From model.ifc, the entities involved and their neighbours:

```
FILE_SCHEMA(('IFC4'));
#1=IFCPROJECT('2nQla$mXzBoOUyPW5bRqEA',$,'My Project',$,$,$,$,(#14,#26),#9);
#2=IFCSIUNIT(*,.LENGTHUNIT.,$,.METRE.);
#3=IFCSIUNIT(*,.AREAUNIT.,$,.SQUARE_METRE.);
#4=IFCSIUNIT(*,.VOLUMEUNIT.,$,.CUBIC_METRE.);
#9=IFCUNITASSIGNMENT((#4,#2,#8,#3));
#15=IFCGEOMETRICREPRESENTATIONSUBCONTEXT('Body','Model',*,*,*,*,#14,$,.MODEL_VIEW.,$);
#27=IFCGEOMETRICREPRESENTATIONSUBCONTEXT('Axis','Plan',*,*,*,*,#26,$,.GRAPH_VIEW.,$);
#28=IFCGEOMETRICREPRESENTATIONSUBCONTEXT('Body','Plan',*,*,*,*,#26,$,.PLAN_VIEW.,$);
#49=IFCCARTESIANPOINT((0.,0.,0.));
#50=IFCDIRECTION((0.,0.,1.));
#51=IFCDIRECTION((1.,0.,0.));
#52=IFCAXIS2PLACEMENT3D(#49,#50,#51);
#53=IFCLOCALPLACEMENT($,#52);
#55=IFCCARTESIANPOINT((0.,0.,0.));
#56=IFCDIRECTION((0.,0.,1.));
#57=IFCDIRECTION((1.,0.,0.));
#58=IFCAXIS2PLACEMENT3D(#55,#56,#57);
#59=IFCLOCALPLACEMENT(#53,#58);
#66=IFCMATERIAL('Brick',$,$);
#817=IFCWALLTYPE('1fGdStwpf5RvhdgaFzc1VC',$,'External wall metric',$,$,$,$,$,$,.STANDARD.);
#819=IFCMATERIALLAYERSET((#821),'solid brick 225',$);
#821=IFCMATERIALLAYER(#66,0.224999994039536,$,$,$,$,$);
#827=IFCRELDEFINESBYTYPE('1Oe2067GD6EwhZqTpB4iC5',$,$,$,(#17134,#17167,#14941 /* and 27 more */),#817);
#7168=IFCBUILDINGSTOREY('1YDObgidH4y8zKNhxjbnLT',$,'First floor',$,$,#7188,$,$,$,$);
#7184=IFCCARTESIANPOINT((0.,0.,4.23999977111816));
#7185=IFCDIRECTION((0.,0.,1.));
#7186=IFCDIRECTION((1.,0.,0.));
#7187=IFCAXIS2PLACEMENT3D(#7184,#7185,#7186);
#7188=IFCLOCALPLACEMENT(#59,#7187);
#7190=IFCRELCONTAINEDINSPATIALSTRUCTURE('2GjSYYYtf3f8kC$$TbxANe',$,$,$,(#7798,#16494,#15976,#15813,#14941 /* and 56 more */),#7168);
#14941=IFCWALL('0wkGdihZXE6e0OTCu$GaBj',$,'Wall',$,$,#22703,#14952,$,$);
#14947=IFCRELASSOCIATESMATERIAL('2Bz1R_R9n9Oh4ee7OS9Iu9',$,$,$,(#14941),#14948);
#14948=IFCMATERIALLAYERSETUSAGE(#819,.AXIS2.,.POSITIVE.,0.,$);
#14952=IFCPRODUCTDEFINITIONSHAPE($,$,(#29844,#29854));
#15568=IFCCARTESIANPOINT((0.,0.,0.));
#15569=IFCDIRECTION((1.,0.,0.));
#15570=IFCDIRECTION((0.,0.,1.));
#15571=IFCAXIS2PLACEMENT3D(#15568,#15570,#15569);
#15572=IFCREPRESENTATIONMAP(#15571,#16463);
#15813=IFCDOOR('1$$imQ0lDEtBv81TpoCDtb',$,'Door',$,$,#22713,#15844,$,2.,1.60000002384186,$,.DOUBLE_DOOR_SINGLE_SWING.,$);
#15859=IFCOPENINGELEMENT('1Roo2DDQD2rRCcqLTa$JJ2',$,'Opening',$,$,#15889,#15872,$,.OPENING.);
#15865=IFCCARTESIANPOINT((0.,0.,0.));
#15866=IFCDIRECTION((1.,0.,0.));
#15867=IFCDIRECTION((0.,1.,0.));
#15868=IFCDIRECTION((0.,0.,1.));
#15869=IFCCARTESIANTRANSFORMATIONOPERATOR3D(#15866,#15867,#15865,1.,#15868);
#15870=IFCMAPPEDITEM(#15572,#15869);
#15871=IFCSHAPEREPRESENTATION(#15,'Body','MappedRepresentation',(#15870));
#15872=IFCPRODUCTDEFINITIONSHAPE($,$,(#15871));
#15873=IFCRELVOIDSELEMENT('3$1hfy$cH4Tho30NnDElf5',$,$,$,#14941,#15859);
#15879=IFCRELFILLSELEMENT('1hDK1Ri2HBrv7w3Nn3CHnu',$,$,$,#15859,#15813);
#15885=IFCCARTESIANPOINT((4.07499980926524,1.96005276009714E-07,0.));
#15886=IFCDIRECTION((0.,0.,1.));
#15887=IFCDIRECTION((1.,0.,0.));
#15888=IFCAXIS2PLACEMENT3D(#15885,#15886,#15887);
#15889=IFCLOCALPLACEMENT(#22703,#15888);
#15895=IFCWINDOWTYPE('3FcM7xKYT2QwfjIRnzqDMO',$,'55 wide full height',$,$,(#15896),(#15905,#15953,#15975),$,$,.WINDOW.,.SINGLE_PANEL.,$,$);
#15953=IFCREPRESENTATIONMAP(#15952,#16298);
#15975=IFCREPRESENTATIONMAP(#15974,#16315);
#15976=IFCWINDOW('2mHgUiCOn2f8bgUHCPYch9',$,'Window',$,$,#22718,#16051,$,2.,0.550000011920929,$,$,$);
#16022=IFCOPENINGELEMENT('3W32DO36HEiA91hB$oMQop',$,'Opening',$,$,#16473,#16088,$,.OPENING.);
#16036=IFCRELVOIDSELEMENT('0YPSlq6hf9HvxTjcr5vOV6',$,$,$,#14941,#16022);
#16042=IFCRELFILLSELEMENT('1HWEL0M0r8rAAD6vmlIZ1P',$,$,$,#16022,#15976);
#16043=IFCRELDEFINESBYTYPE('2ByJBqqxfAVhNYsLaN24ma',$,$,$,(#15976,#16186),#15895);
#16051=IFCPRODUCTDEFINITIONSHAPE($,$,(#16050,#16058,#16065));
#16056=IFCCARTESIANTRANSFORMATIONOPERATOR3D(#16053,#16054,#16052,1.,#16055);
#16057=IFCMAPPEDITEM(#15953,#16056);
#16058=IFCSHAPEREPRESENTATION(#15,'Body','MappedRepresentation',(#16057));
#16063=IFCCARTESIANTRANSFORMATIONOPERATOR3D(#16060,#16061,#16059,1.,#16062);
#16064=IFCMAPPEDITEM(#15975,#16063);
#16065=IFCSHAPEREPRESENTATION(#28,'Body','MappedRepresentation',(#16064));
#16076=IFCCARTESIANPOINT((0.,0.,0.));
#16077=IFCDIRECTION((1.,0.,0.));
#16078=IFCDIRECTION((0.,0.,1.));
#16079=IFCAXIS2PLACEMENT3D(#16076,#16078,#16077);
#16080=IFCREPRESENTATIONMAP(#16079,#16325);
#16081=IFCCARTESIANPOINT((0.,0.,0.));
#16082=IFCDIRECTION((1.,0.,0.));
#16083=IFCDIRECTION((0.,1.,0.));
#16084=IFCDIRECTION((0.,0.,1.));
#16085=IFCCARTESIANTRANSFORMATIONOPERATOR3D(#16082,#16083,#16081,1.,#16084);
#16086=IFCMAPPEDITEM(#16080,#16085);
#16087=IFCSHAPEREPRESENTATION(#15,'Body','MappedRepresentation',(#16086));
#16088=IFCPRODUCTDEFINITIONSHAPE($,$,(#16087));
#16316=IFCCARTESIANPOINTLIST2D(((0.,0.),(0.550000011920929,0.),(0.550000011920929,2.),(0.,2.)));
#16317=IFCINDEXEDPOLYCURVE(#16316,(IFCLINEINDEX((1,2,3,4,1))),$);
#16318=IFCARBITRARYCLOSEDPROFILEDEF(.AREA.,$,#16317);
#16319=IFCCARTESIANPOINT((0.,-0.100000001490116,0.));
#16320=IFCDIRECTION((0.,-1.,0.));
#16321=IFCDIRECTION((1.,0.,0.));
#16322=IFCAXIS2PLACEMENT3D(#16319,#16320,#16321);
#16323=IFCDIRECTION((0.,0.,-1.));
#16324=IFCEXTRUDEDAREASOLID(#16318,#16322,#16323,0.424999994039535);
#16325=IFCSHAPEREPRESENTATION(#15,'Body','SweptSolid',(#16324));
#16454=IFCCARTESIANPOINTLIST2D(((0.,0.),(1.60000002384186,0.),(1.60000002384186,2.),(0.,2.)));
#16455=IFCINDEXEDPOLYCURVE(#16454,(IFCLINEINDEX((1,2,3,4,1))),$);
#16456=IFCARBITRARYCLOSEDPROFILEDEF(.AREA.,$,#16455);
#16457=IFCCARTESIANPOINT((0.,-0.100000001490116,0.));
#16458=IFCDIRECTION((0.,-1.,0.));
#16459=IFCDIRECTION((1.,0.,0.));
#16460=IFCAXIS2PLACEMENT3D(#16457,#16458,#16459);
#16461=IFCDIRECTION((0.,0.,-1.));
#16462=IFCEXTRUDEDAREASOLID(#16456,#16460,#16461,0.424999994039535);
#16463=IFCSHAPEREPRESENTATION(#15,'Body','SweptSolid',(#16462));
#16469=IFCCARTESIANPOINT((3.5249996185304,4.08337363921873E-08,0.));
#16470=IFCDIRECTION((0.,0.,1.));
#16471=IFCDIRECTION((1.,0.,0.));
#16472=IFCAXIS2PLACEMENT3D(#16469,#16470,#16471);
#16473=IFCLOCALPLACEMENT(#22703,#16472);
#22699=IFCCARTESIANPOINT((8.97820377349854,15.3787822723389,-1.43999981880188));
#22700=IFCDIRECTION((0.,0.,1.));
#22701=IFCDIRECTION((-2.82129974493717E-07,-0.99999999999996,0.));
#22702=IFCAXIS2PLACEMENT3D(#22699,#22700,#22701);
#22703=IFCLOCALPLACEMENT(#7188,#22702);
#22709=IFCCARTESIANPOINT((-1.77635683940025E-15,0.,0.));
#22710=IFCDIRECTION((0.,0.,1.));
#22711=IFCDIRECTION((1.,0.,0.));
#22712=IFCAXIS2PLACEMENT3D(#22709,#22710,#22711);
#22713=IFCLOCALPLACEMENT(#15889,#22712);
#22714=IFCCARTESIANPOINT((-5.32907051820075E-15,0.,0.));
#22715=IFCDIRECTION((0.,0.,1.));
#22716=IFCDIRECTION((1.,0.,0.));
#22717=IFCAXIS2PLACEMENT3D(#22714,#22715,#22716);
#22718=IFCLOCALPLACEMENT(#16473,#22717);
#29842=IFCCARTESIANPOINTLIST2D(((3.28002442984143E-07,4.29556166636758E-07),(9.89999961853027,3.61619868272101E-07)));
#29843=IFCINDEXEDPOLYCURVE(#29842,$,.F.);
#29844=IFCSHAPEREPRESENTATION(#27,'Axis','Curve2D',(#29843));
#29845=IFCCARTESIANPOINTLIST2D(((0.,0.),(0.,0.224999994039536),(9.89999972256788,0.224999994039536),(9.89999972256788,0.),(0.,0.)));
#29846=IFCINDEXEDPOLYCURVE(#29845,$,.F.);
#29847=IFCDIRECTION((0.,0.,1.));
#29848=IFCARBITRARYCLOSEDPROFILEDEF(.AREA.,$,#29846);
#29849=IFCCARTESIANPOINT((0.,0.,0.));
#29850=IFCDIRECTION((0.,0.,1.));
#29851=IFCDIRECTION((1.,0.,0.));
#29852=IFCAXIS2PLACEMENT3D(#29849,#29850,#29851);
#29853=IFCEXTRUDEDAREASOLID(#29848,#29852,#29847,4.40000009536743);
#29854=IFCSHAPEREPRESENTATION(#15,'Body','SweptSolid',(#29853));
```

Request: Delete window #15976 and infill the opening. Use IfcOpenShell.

```python
import ifcopenshell
import ifcopenshell.api.feature
import ifcopenshell.api.root
import ifcopenshell.geom
import ifcopenshell.util.shape

model = ifcopenshell.open("model.ifc")
settings = ifcopenshell.geom.settings()


def volume(element):
    """Net volume in cubic metres, openings subtracted."""
    shape = ifcopenshell.geom.create_shape(settings, element)
    return ifcopenshell.util.shape.get_volume(shape.geometry)


window = model.by_guid("2mHgUiCOn2f8bgUHCPYch9")
opening = window.FillsVoids[0].RelatingOpeningElement
wall = opening.VoidsElements[0].RelatingBuildingElement
before = volume(wall)

ifcopenshell.api.root.remove_product(model, product=window)
ifcopenshell.api.feature.remove_feature(model, feature=opening)

after = volume(wall)

print(f"wall volume {before:.3f} -> {after:.3f} m3")

model.write("model-out.ifc")
```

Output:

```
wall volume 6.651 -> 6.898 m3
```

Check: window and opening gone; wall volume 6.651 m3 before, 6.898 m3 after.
